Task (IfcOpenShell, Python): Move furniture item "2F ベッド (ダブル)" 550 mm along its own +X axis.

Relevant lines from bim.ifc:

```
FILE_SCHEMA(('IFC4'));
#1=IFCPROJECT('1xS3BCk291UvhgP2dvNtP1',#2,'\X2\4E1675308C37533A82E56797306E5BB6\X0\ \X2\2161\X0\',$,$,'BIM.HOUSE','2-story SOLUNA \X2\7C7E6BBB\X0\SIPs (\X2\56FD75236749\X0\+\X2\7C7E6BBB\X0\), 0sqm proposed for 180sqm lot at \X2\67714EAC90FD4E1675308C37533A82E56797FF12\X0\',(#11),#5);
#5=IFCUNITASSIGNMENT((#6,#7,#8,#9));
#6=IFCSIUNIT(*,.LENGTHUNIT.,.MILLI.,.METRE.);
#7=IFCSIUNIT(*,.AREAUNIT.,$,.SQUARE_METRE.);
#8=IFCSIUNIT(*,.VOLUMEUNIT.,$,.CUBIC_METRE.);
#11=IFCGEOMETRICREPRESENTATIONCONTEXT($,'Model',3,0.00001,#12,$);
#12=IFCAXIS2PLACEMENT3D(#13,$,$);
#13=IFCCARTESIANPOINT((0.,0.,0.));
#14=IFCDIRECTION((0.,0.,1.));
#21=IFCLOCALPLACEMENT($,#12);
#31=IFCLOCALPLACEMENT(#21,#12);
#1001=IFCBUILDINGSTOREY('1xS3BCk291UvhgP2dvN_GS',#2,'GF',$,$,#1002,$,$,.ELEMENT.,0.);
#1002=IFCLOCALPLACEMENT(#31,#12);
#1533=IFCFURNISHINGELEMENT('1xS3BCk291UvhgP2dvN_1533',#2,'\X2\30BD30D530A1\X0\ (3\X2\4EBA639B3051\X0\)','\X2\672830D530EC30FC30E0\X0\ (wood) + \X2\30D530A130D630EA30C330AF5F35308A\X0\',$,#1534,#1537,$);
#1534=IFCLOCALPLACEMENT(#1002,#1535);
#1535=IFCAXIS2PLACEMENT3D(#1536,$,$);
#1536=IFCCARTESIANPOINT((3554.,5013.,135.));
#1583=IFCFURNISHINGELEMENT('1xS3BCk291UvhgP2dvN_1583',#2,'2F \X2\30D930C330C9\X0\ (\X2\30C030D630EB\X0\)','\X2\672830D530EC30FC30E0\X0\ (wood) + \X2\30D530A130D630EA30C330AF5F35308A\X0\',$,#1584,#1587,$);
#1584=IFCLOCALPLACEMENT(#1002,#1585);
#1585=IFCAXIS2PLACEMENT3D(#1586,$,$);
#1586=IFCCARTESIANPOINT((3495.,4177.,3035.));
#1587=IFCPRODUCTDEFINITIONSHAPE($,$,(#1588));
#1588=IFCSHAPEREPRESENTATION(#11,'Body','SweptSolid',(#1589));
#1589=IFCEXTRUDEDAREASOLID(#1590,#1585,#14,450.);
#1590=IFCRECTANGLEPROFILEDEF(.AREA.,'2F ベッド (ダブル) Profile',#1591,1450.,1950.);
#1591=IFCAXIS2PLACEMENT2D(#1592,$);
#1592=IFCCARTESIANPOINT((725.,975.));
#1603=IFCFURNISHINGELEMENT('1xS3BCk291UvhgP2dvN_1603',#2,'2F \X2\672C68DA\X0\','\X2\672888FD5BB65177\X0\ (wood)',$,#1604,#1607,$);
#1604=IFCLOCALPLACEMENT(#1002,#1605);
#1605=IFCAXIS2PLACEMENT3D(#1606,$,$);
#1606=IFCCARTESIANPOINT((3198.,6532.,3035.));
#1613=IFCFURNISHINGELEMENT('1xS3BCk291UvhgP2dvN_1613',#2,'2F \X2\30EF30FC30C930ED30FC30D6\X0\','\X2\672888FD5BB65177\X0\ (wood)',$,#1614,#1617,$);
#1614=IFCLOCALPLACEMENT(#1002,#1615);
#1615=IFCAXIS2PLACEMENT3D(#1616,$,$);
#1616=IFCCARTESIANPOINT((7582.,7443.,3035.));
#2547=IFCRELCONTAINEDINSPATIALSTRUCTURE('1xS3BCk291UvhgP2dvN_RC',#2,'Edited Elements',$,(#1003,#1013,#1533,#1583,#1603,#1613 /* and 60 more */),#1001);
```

```python
import ifcopenshell
import ifcopenshell.api.geometry
import ifcopenshell.util.placement

model = ifcopenshell.open("bim.ifc")

item = model.by_id(1583)
matrix = ifcopenshell.util.placement.get_local_placement(item.ObjectPlacement)
matrix[:3, 3] += matrix[:3, 0] * 550.0
ifcopenshell.api.geometry.edit_object_placement(model, product=item, matrix=matrix, is_si=False)

print(ifcopenshell.util.placement.get_local_placement(item.ObjectPlacement).round(3) + 0.0)

model.write("bim-out.ifc")
```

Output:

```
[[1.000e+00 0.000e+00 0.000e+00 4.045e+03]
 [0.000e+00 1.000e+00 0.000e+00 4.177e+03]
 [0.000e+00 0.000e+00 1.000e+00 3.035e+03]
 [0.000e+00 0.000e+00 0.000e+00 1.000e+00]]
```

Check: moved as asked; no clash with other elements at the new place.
